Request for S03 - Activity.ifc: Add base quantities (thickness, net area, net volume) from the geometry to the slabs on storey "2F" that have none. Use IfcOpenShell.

First a look at what the model holds.

```python
import ifcopenshell
import ifcopenshell.util.element
import ifcopenshell.util.unit

model = ifcopenshell.open("S03 - Activity.ifc")
print(model.schema)
for unit_type in ("LENGTHUNIT", "AREAUNIT", "VOLUMEUNIT"):
    print(unit_type, ifcopenshell.util.unit.calculate_unit_scale(model, unit_type))
storey = next(s for s in model.by_type("IfcBuildingStorey") if s.Name == "2F")
slabs = [e for e in ifcopenshell.util.element.get_decomposition(storey) if e.is_a("IfcSlab")]
for e in sorted(slabs, key=lambda e: e.id()):
    print(e.id(), e.is_a(), e.Name, list(ifcopenshell.util.element.get_psets(e, qtos_only=True)), sep=" | ")
```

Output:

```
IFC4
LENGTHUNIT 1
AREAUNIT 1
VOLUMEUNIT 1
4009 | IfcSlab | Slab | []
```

```python
import ifcopenshell
import ifcopenshell.api.pset
import ifcopenshell.geom
import ifcopenshell.util.element
import ifcopenshell.util.shape
import ifcopenshell.util.unit

model = ifcopenshell.open("S03 - Activity.ifc")
unit_scale = ifcopenshell.util.unit.calculate_unit_scale(model)
area_scale = ifcopenshell.util.unit.calculate_unit_scale(model, "AREAUNIT")
volume_scale = ifcopenshell.util.unit.calculate_unit_scale(model, "VOLUMEUNIT")
settings = ifcopenshell.geom.settings()

storey = next(s for s in model.by_type("IfcBuildingStorey") if s.Name == "2F")
slabs = [e for e in ifcopenshell.util.element.get_decomposition(storey) if e.is_a("IfcSlab")]

for e in sorted(slabs, key=lambda e: e.id()):
    if ifcopenshell.util.element.get_psets(e, qtos_only=True, should_inherit=False):
        continue
    # Geometry comes back in metres, in the element's own axes.
    shape = ifcopenshell.geom.create_shape(settings, e)
    values = {
        "Width": ifcopenshell.util.shape.get_z(shape.geometry) / unit_scale,
        "NetArea": ifcopenshell.util.shape.get_footprint_area(shape.geometry) / area_scale,
        "NetVolume": ifcopenshell.util.shape.get_volume(shape.geometry) / volume_scale,
    }
    qto = ifcopenshell.api.pset.add_qto(model, product=e, name="Qto_SlabBaseQuantities")
    ifcopenshell.api.pset.edit_qto(model, qto=qto, properties=values)
    print(e.id(), {k: round(v, 3) for k, v in values.items()})

model.write("S03 - Activity_updated.ifc")
```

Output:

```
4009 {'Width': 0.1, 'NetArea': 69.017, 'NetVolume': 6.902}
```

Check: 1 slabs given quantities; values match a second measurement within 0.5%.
